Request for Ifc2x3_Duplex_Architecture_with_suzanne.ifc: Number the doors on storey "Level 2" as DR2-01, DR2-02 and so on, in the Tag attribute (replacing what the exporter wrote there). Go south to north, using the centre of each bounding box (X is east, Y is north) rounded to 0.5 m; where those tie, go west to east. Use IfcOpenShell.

First a look at what the model holds.

```python
import ifcopenshell
import ifcopenshell.util.element
import ifcopenshell.util.placement

model = ifcopenshell.open("Ifc2x3_Duplex_Architecture_with_suzanne.ifc")
print(model.schema)
storey = next(s for s in model.by_type("IfcBuildingStorey") if s.Name == "Level 2")
doors = [e for e in ifcopenshell.util.element.get_decomposition(storey) if e.is_a("IfcDoor")]
for e in sorted(doors, key=lambda e: e.id()):
    origin = ifcopenshell.util.placement.get_local_placement(e.ObjectPlacement)[:3, 3]
    print(e.id(), e.Tag, e.Name, origin.round(2) + 0.0, sep=" | ")
```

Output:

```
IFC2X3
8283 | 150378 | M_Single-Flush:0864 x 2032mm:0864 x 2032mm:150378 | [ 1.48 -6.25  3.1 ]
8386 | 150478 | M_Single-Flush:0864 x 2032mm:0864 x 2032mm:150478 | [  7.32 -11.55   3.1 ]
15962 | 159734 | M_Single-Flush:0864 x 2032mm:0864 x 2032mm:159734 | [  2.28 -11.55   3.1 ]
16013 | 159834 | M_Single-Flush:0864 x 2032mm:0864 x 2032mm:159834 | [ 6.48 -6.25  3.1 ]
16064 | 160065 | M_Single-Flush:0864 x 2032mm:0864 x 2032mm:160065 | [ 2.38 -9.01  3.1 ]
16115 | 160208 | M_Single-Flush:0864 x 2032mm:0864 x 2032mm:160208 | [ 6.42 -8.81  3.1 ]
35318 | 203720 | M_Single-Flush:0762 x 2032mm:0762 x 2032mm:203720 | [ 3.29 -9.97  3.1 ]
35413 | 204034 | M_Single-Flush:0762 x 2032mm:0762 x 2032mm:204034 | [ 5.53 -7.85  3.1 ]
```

```python
import ifcopenshell
import ifcopenshell.geom
import ifcopenshell.util.element
import ifcopenshell.util.shape

model = ifcopenshell.open("Ifc2x3_Duplex_Architecture_with_suzanne.ifc")
settings = ifcopenshell.geom.settings()
settings.set("use-world-coords", True)


def centre(element):
    shape = ifcopenshell.geom.create_shape(settings, element)
    return ifcopenshell.util.shape.get_bbox_centroid(shape.geometry)


storey = next(s for s in model.by_type("IfcBuildingStorey") if s.Name == "Level 2")
doors = [e for e in ifcopenshell.util.element.get_decomposition(storey) if e.is_a("IfcDoor")]

# Insertion points can sit at a corner or the storey origin, so sort by the geometry (in metres).
centres = {e: centre(e) for e in doors}
doors.sort(key=lambda e: (round(centres[e][1] / 0.5), centres[e][0]))

for i, e in enumerate(doors, start=1):
    number = f"DR2-{i:02d}"
    e.Tag = number
    print(e.id(), number)

model.write("Ifc2x3_Duplex_Architecture_with_suzanne_updated.ifc")
```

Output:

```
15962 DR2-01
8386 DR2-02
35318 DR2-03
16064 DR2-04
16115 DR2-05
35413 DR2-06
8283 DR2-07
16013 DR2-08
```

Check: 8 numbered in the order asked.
